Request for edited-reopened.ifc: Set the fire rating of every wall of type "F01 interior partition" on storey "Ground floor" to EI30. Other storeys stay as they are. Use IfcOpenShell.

First a look at what the model holds.

```python
import ifcopenshell
import ifcopenshell.util.element

model = ifcopenshell.open("edited-reopened.ifc")
print(model.schema)
storey = next(s for s in model.by_type("IfcBuildingStorey") if s.Name == "Ground floor")
walls = [e for e in ifcopenshell.util.element.get_decomposition(storey) if e.is_a("IfcWall")]
seen = {}
for e in walls:
    element_type = ifcopenshell.util.element.get_type(e)
    key = (element_type.Name if element_type != e and element_type else None, ifcopenshell.util.element.get_pset(e, "Pset_WallCommon", "FireRating"))
    seen[key] = seen.get(key, 0) + 1
for (name, value), count in sorted(seen.items(), key=str):
    print(count, "x", name, "|", value)
```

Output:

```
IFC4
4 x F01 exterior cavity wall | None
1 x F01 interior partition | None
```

```python
import ifcopenshell
import ifcopenshell.api.pset
import ifcopenshell.util.element

model = ifcopenshell.open("edited-reopened.ifc")

storey = next(s for s in model.by_type("IfcBuildingStorey") if s.Name == "Ground floor")
walls = [e for e in ifcopenshell.util.element.get_decomposition(storey) if e.is_a("IfcWall")]

count = 0
for e in walls:
    element_type = ifcopenshell.util.element.get_type(e)
    if element_type in (None, e) or element_type.Name != "F01 interior partition":
        continue
    # add_pset returns the element's existing set when there is one.
    pset = ifcopenshell.api.pset.add_pset(model, product=e, name="Pset_WallCommon")
    ifcopenshell.api.pset.edit_pset(model, pset=pset, properties={"FireRating": "EI30"})
    count += 1

print(count, "walls updated")

model.write("edited-reopened_updated.ifc")
```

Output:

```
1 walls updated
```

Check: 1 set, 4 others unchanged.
